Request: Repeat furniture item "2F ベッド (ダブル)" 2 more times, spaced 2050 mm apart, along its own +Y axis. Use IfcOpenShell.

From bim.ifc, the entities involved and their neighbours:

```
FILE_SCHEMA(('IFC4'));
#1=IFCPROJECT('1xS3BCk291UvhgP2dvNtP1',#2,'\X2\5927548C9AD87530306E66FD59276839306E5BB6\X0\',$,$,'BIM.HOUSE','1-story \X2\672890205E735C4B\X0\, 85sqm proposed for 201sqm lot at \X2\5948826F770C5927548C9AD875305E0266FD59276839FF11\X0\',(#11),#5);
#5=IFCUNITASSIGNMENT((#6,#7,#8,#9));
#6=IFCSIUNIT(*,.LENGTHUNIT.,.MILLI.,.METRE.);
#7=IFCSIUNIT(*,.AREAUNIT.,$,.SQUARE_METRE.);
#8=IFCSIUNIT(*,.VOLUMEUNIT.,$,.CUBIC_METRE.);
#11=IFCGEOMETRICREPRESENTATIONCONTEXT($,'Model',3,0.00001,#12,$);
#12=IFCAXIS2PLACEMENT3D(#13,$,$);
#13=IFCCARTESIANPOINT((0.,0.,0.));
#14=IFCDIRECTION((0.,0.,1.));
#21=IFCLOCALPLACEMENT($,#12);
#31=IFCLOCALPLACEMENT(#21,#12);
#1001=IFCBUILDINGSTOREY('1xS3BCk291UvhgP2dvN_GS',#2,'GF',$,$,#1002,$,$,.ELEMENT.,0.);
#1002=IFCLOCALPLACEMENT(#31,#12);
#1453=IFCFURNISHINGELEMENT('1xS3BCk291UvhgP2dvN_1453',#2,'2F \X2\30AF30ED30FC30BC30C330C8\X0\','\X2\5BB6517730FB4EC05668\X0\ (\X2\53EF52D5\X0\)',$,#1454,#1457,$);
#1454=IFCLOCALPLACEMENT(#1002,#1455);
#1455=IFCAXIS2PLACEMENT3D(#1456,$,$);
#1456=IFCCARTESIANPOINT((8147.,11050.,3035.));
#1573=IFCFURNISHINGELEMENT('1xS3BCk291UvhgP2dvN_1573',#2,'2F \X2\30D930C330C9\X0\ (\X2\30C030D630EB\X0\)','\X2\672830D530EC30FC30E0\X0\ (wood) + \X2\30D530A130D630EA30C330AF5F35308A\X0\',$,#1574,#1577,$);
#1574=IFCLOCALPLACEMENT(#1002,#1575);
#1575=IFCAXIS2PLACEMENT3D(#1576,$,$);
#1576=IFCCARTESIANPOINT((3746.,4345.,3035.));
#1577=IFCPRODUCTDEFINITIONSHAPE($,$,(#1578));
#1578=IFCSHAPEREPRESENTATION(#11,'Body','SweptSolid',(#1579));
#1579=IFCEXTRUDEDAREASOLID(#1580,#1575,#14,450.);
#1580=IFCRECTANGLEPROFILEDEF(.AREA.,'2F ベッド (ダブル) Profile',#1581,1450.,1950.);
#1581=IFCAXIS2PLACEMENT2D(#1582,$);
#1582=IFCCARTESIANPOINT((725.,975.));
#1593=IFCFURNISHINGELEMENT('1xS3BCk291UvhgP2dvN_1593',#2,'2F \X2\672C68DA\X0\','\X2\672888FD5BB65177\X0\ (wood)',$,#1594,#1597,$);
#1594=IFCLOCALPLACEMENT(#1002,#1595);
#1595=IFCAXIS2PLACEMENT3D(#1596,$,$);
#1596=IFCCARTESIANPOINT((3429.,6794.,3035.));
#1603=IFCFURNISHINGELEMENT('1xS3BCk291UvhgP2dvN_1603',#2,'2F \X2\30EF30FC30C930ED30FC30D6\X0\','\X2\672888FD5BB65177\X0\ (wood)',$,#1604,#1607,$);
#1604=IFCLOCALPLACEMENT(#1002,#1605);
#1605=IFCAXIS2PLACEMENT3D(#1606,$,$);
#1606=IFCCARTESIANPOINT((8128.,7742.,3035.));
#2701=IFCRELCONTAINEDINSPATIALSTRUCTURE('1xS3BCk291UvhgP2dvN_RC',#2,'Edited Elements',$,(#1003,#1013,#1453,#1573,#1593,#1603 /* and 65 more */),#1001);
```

```python
import ifcopenshell
import ifcopenshell.api.geometry
import ifcopenshell.api.root
import ifcopenshell.util.element
import ifcopenshell.util.placement
import ifcopenshell.util.unit

model = ifcopenshell.open("bim.ifc")
unit_scale = ifcopenshell.util.unit.calculate_unit_scale(model)


def reuse_history(source, copy):
    """copy_class also copies each property set's owner history, people and application; keep the originals."""
    for rel in copy.IsDefinedBy:
        if rel.is_a("IfcRelDefinesByProperties") and (history := rel.RelatingPropertyDefinition.OwnerHistory):
            rel.RelatingPropertyDefinition.OwnerHistory = source.OwnerHistory
            ifcopenshell.util.element.remove_deep2(model, history)


source = model.by_id(1573)
base = ifcopenshell.util.placement.get_local_placement(source.ObjectPlacement)
step = base[:3, 1] * 2.05 / unit_scale

for i in range(1, 3):
    copy = ifcopenshell.api.root.copy_class(model, product=source)
    copy.Representation = ifcopenshell.util.element.copy_deep(
        model, source.Representation, exclude=["IfcGeometricRepresentationContext", "IfcRepresentationMap"]
    )
    reuse_history(source, copy)
    matrix = base.copy()
    matrix[:3, 3] += i * step
    print("added at", matrix[:3, 3].round(3) + 0.0)
    ifcopenshell.api.geometry.edit_object_placement(model, product=copy, matrix=matrix, is_si=False)

model.write("bim_rev.ifc")
```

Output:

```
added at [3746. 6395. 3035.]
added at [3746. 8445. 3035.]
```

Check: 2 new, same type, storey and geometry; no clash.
